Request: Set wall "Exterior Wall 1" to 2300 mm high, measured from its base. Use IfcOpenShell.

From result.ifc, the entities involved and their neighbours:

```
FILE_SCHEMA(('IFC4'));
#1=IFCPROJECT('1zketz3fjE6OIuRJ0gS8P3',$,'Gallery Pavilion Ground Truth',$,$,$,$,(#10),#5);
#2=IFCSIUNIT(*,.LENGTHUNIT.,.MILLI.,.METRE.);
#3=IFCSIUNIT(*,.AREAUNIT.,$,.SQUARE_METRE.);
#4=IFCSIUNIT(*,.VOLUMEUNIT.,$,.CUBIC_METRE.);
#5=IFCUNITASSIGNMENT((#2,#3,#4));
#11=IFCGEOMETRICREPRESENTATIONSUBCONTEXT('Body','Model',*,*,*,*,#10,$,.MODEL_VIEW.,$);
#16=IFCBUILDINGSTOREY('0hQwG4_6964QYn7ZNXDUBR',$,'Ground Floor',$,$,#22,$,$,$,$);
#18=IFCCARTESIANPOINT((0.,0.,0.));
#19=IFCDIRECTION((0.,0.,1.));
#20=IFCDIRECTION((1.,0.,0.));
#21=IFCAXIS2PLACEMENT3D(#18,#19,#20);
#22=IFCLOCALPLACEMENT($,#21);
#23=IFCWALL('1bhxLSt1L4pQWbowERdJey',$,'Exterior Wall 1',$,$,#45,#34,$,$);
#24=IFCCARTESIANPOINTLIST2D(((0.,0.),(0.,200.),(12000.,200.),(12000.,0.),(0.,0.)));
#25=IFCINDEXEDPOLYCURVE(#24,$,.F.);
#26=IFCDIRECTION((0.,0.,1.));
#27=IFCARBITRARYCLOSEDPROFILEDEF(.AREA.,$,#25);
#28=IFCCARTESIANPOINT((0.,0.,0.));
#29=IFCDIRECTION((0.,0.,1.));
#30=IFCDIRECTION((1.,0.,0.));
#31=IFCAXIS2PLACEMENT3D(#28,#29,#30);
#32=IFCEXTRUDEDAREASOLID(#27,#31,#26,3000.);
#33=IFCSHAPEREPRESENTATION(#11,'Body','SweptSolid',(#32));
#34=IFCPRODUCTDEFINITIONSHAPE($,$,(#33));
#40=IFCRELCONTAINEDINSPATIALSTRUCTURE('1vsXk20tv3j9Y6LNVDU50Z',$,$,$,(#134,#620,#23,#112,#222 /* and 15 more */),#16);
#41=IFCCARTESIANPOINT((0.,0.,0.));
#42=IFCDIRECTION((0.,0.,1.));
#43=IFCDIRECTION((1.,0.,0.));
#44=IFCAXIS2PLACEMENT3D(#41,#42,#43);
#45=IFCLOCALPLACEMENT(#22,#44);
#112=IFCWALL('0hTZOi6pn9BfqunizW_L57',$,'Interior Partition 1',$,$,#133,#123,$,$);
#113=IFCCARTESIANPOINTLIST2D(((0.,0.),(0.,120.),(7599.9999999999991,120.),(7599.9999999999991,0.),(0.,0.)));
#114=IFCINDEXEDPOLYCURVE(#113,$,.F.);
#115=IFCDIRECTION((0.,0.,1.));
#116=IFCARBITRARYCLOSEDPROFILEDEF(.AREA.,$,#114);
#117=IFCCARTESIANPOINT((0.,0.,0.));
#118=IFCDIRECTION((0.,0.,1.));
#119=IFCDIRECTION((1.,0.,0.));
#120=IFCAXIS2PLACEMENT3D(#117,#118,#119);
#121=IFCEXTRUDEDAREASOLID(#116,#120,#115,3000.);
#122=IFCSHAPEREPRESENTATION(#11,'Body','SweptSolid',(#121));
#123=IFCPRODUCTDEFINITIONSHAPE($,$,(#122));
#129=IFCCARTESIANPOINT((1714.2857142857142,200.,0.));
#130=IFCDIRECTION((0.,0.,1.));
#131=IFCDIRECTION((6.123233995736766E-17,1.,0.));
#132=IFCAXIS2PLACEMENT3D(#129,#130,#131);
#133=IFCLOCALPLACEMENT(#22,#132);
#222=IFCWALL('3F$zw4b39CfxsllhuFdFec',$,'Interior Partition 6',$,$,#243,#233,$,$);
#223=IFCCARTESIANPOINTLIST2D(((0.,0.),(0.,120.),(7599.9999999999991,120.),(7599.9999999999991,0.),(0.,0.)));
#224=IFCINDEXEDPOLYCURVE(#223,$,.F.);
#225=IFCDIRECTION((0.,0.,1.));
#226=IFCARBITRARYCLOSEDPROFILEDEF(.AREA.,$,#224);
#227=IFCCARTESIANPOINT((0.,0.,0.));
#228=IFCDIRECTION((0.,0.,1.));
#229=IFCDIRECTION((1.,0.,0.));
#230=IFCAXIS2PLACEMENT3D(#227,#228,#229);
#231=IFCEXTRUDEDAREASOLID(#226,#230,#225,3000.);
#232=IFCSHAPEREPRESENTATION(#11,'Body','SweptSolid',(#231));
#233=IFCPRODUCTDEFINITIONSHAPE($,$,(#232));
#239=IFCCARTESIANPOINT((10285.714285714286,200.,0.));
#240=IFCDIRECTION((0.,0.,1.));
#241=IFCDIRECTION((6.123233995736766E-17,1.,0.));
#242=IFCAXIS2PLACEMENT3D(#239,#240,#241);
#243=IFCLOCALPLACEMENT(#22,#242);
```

```python
import ifcopenshell
import ifcopenshell.geom
import ifcopenshell.util.representation
import ifcopenshell.util.shape
import ifcopenshell.util.unit

model = ifcopenshell.open("result.ifc")
unit_scale = ifcopenshell.util.unit.calculate_unit_scale(model)
settings = ifcopenshell.geom.settings()


def volume(element):
    """Net volume in cubic metres, openings subtracted."""
    shape = ifcopenshell.geom.create_shape(settings, element)
    return ifcopenshell.util.shape.get_volume(shape.geometry)


wall = model.by_guid("1bhxLSt1L4pQWbowERdJey")
before = volume(wall)

body = ifcopenshell.util.representation.get_representation(wall, "Model", "Body")
solid = body.Items[0]
old_height = solid.Depth
solid.Depth = 2.3 / unit_scale
after = volume(wall)

print(f"height {old_height:g} -> {solid.Depth:g}, volume {before:.3f} -> {after:.3f} m3")

model.write("result_rev.ifc")
```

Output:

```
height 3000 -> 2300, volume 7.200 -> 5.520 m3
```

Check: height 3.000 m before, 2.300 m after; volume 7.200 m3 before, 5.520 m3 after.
